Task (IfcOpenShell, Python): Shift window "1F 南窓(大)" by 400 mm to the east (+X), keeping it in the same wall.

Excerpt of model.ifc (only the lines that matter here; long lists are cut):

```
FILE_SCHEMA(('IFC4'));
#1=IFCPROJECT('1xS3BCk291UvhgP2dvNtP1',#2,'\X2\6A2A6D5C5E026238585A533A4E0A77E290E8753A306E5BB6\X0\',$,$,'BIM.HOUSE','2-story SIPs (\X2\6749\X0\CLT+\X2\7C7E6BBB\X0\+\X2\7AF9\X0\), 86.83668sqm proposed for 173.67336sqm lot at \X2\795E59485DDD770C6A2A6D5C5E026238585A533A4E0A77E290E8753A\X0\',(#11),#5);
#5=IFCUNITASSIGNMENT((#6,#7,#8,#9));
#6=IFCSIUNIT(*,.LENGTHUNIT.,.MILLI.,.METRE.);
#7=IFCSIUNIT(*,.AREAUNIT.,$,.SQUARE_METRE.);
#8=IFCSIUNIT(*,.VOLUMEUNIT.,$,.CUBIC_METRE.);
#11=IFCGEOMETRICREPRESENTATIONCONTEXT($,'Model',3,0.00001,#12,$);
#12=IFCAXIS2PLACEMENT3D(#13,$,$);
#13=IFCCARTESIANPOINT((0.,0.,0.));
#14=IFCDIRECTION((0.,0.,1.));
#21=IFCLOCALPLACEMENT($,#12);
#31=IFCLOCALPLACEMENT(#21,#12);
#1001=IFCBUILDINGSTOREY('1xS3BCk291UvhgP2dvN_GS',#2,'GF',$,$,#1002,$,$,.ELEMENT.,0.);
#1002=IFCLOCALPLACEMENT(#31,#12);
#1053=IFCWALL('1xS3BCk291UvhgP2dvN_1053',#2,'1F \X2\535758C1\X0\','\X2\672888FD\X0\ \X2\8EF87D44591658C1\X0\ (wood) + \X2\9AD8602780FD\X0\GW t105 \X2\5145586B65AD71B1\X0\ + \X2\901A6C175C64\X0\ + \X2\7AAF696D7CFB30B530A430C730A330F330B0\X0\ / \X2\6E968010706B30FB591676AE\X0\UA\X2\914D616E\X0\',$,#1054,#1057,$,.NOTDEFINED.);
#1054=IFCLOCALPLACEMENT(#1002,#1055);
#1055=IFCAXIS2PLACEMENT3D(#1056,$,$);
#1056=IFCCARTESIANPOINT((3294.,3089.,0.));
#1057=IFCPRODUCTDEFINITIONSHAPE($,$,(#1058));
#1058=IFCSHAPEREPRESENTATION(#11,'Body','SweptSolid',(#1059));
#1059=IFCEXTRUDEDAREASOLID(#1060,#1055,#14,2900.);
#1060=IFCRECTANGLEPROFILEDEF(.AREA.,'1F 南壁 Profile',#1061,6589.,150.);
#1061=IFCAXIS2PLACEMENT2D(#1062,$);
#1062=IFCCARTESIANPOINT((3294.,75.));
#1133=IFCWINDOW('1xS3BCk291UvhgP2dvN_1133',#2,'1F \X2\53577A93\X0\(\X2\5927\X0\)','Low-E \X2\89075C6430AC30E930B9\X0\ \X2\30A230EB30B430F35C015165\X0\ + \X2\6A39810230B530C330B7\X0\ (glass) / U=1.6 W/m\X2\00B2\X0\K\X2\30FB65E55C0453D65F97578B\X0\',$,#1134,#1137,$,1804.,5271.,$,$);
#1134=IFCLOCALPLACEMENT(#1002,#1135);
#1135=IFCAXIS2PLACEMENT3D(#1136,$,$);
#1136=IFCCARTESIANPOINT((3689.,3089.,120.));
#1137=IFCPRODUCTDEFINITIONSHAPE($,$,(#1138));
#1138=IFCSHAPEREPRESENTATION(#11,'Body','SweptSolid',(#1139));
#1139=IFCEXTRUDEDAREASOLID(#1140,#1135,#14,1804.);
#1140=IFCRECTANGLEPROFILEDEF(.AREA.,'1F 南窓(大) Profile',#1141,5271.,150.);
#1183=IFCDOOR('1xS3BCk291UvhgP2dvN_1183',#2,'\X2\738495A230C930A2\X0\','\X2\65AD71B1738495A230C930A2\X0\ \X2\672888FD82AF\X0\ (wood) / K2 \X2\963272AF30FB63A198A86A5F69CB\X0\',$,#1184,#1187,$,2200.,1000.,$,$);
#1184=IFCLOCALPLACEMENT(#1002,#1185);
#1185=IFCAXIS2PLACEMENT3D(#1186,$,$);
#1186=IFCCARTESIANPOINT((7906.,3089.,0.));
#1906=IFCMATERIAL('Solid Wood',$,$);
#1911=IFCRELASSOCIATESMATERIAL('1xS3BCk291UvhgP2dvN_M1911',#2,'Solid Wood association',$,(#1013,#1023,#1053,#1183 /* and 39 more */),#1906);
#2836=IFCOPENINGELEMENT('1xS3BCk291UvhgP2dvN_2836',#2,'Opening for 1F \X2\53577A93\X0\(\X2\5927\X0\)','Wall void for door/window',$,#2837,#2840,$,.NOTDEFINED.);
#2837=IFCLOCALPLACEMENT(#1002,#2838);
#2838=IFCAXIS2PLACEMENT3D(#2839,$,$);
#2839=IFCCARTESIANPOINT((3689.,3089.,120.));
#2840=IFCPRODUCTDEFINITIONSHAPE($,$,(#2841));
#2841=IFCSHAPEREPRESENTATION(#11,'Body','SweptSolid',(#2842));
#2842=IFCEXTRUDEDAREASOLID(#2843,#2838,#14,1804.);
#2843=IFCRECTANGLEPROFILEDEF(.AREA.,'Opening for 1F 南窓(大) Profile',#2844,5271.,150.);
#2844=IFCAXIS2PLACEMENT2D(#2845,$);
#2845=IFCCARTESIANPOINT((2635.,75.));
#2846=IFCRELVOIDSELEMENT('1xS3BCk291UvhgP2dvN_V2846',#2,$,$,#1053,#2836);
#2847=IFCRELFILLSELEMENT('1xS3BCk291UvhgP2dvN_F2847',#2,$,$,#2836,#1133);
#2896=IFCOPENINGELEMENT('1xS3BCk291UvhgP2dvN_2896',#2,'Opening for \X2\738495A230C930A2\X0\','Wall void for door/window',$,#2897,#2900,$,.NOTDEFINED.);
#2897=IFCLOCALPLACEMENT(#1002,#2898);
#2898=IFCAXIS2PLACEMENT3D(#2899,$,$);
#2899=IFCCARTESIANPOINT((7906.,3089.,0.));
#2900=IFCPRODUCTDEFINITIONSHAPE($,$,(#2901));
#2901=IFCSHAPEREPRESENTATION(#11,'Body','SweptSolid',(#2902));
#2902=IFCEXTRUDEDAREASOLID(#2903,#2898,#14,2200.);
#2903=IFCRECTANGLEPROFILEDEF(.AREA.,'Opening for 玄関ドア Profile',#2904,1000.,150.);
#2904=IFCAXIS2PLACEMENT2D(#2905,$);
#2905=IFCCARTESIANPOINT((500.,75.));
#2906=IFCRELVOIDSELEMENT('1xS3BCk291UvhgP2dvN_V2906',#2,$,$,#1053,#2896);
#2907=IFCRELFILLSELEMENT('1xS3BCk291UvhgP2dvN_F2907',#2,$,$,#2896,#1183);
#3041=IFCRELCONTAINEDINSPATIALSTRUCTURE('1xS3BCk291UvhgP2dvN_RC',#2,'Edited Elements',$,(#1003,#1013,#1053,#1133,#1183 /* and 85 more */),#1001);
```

```python
import ifcopenshell
import ifcopenshell.api.geometry
import ifcopenshell.util.placement

model = ifcopenshell.open("model.ifc")

window = model.by_guid("1xS3BCk291UvhgP2dvN_1133")
opening = window.FillsVoids[0].RelatingOpeningElement
wall = opening.VoidsElements[0].RelatingBuildingElement

wall_matrix = ifcopenshell.util.placement.get_local_placement(wall.ObjectPlacement)
shift = wall_matrix[:3, 0] * 400.0
before = ifcopenshell.util.placement.get_local_placement(window.ObjectPlacement)[:3, 3].copy()

# The window is not placed relative to its opening, so move both.
for product in (opening, window):
    matrix = ifcopenshell.util.placement.get_local_placement(product.ObjectPlacement)
    matrix[:3, 3] += shift
    ifcopenshell.api.geometry.edit_object_placement(model, product=product, matrix=matrix, is_si=False)

after = ifcopenshell.util.placement.get_local_placement(window.ObjectPlacement)[:3, 3]
print("window moved by", (after - before).round(3) + 0.0)

model.write("model_updated.ifc")
```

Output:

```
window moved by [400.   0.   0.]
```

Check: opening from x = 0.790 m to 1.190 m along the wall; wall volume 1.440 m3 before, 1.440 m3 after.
